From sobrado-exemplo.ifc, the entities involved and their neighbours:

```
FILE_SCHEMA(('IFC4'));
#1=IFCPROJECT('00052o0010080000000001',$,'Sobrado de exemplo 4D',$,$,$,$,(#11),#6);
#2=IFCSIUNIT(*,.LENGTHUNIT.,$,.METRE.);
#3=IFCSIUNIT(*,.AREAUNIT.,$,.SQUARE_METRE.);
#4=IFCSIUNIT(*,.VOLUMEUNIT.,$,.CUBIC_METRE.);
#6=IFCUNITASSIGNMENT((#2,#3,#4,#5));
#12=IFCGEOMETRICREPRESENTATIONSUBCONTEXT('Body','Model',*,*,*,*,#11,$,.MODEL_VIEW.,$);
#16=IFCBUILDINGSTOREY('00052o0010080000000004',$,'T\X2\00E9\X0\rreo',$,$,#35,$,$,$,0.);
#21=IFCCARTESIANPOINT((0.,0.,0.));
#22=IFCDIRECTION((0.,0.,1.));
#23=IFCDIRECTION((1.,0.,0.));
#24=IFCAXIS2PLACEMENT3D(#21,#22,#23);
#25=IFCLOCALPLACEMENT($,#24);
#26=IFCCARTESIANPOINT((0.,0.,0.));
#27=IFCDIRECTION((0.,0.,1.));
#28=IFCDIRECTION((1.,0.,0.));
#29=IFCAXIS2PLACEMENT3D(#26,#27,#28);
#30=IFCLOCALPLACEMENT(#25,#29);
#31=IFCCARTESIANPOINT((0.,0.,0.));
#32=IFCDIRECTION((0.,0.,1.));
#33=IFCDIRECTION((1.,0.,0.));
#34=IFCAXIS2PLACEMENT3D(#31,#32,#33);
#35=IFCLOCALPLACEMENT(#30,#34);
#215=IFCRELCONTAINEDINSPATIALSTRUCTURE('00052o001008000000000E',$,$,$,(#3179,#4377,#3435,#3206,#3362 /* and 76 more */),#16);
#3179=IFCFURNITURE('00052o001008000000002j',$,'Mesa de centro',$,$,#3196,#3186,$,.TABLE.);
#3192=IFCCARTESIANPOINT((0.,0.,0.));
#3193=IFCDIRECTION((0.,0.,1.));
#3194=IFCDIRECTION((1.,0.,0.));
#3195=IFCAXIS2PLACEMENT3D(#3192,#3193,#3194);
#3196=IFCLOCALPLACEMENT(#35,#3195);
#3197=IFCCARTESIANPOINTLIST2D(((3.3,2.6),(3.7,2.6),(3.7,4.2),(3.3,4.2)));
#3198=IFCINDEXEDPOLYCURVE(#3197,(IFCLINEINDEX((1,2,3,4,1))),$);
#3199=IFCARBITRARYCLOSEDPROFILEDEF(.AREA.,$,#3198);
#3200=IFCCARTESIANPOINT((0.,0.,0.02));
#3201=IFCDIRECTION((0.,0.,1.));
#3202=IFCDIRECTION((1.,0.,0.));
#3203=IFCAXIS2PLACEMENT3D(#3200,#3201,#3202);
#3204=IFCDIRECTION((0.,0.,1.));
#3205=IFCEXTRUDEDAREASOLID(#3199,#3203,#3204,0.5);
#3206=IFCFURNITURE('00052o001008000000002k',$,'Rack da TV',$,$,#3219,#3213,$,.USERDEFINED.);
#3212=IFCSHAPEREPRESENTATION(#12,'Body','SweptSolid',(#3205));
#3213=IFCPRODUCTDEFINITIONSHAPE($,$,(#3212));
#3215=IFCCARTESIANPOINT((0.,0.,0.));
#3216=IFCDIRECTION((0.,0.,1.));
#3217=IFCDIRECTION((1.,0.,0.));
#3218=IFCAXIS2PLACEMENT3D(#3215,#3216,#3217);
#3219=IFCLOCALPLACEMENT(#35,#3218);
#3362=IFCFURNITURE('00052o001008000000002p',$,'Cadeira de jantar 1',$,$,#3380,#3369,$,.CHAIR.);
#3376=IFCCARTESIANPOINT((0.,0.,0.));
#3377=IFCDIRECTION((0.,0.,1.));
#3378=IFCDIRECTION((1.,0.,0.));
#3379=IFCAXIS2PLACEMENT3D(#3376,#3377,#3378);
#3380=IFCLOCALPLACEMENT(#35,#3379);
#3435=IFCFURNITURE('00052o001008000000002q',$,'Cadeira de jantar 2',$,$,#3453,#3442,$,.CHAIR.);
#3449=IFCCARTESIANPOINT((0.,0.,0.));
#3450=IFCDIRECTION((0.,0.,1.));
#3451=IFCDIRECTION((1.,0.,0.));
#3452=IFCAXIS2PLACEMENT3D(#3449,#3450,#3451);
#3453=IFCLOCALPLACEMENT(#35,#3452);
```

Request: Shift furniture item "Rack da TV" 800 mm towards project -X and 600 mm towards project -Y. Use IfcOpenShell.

```python
import ifcopenshell
import ifcopenshell.api.geometry
import ifcopenshell.util.placement
import ifcopenshell.util.unit

model = ifcopenshell.open("sobrado-exemplo.ifc")
unit_scale = ifcopenshell.util.unit.calculate_unit_scale(model)

item = model.by_guid("00052o001008000000002k")
matrix = ifcopenshell.util.placement.get_local_placement(item.ObjectPlacement)
matrix[0, 3] -= 0.8 / unit_scale
matrix[1, 3] -= 0.6 / unit_scale
ifcopenshell.api.geometry.edit_object_placement(model, product=item, matrix=matrix, is_si=False)

print(ifcopenshell.util.placement.get_local_placement(item.ObjectPlacement).round(3) + 0.0)

model.write("sobrado-exemplo_edited.ifc")
```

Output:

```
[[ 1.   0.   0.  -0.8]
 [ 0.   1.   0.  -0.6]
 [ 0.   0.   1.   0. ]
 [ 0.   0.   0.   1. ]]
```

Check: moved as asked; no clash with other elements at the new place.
